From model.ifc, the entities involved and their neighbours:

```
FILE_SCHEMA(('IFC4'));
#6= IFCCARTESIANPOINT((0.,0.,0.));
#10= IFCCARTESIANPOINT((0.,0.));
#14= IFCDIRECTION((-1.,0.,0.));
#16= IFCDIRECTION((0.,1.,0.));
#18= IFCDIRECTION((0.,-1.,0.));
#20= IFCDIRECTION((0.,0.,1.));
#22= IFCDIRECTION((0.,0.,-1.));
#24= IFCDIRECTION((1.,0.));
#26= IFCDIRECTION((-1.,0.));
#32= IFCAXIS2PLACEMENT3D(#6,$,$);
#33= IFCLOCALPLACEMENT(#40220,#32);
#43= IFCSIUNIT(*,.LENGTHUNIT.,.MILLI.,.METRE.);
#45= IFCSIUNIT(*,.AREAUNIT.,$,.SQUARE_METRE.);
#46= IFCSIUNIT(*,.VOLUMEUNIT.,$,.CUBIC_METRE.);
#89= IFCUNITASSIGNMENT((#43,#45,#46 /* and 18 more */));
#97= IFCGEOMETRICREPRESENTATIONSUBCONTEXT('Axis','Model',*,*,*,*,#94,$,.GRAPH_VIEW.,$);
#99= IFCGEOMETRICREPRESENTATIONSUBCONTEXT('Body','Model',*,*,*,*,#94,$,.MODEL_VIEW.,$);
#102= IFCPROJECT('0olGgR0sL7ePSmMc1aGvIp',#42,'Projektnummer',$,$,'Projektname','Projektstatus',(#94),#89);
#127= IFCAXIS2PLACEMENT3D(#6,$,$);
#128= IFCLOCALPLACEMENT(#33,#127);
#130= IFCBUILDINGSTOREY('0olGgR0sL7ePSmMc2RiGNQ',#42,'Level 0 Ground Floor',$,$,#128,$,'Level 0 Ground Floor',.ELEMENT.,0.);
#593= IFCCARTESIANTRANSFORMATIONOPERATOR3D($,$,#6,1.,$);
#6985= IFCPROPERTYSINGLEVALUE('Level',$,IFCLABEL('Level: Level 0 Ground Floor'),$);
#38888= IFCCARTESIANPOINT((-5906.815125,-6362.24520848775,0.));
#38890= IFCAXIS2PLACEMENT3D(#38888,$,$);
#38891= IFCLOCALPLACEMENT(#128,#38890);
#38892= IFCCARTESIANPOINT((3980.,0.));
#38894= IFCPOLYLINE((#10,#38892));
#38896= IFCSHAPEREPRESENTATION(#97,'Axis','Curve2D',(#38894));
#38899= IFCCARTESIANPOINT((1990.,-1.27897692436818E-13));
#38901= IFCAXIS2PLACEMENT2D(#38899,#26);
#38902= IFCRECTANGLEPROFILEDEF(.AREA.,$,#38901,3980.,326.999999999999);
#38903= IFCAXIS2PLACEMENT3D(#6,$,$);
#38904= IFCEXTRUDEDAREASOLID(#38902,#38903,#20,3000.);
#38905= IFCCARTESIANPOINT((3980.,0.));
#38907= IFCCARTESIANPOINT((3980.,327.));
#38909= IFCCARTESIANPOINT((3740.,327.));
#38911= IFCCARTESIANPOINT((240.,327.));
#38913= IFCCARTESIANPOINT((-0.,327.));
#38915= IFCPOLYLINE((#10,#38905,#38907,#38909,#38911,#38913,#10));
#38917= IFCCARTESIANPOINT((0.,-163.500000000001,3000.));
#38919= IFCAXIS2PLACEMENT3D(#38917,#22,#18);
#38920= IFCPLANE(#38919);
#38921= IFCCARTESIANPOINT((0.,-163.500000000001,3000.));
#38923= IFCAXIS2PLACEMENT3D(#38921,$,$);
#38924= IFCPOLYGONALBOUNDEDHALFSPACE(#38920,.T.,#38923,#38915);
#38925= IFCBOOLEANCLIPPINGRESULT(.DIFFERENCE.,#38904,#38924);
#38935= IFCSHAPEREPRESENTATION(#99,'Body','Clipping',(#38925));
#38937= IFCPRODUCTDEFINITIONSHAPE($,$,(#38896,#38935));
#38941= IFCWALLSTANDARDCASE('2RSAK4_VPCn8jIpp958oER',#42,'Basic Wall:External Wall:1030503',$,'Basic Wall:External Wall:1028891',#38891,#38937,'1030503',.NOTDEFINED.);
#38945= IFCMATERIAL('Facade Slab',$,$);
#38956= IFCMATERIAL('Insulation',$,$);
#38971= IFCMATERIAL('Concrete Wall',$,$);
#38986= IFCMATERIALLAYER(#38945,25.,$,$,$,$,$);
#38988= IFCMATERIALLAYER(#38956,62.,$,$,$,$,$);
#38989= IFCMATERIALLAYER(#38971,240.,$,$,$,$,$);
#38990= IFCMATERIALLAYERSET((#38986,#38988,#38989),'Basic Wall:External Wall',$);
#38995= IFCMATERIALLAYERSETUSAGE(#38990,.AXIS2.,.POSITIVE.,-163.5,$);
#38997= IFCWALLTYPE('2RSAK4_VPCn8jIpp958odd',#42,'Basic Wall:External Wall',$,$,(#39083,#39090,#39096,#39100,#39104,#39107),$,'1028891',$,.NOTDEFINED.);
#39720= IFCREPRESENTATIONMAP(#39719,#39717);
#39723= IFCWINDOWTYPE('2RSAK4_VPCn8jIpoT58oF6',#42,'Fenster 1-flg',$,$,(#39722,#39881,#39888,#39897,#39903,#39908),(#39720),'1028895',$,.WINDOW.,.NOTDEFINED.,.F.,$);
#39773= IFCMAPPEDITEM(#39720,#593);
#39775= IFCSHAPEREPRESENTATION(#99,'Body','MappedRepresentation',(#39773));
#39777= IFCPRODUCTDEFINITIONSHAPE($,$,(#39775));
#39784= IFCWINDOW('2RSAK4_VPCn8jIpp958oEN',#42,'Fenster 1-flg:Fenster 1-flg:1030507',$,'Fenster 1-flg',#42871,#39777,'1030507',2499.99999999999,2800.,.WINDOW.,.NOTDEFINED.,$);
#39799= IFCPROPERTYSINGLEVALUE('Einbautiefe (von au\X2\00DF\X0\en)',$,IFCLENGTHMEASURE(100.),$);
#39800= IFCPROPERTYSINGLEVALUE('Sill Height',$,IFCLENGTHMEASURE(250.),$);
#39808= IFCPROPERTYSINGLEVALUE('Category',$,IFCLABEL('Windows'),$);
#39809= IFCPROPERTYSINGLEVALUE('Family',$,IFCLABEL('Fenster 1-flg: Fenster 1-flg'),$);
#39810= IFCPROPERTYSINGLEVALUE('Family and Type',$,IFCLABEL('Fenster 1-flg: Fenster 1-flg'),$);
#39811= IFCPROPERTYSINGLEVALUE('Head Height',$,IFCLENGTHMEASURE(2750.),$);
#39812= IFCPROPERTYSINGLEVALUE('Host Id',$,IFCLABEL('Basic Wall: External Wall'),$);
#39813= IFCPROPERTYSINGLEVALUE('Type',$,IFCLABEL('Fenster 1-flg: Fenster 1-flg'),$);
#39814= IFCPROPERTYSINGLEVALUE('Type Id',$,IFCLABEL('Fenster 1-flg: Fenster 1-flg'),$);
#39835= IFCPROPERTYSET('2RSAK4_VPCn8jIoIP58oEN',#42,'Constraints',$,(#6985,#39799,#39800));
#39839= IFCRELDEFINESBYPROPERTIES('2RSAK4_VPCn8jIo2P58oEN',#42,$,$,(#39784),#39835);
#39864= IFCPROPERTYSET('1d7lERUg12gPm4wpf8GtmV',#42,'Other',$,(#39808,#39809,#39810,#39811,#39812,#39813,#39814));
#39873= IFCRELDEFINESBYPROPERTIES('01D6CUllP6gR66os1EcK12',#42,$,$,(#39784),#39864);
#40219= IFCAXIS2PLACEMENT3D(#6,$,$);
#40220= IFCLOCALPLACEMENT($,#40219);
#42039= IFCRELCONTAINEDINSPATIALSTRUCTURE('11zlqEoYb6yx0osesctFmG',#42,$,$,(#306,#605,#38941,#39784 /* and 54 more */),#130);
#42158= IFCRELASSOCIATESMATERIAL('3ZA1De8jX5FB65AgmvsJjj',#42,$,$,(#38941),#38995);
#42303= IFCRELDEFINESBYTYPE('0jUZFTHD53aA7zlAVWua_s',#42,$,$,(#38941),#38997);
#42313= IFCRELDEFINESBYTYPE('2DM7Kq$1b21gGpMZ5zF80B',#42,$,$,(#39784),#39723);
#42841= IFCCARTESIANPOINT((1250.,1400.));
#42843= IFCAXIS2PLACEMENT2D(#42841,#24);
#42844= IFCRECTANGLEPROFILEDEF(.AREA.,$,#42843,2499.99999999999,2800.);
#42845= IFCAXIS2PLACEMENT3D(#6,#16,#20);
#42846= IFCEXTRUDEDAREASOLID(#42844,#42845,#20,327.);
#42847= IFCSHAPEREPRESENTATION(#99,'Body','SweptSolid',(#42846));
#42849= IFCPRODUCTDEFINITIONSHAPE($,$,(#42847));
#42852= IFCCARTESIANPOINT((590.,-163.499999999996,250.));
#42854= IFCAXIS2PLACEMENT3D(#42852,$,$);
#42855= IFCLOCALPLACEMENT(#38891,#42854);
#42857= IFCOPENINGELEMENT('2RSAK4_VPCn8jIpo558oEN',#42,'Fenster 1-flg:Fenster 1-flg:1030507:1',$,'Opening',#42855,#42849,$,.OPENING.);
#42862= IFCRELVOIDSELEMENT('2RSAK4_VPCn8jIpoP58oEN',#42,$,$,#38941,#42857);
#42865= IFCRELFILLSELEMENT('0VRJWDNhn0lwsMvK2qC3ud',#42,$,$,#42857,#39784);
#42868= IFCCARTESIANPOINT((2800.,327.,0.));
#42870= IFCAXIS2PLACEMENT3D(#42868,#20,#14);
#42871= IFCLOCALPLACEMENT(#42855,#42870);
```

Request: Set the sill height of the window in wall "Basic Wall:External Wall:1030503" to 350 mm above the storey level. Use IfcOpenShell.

```python
import numpy as np
import ifcopenshell
import ifcopenshell.api.geometry
import ifcopenshell.api.pset
import ifcopenshell.geom
import ifcopenshell.util.element
import ifcopenshell.util.placement
import ifcopenshell.util.shape
import ifcopenshell.util.unit

model = ifcopenshell.open("model.ifc")
unit_scale = ifcopenshell.util.unit.calculate_unit_scale(model)

window = model.by_guid("2RSAK4_VPCn8jIpp958oEN")
opening = window.FillsVoids[0].RelatingOpeningElement
storey = ifcopenshell.util.element.get_container(window, ifc_class="IfcBuildingStorey")
level = ifcopenshell.util.placement.get_local_placement(storey.ObjectPlacement)[2, 3]

# The opening's origin need not be at the sill, so measure its lowest point.
shape = ifcopenshell.geom.create_shape(ifcopenshell.geom.settings(), opening)
bottom = ifcopenshell.util.shape.get_shape_bottom_elevation(shape, shape.geometry) / unit_scale
dz = level + 0.35 / unit_scale - bottom

shift = np.array([0.0, 0.0, dz])
# The window is placed relative to its opening, so it follows when the opening moves.
matrix = ifcopenshell.util.placement.get_local_placement(opening.ObjectPlacement)
matrix[:3, 3] += shift
ifcopenshell.api.geometry.edit_object_placement(
    model, product=opening, matrix=matrix, is_si=False, should_transform_children=True
)

# Keep the stored heights in step.
pset = model.by_id(ifcopenshell.util.element.get_pset(window, "Constraints", should_inherit=False)["id"])
ifcopenshell.api.pset.edit_pset(model, pset=pset, properties={
    "Sill Height": model.create_entity("IfcLengthMeasure", ifcopenshell.util.element.get_pset(window, "Constraints", "Sill Height") + dz),
})
pset = model.by_id(ifcopenshell.util.element.get_pset(window, "Other", should_inherit=False)["id"])
ifcopenshell.api.pset.edit_pset(model, pset=pset, properties={
    "Head Height": model.create_entity("IfcLengthMeasure", ifcopenshell.util.element.get_pset(window, "Other", "Head Height") + dz),
})

print(f"moved by {dz * unit_scale:+.3f} m")

model.write("model_updated.ifc")
```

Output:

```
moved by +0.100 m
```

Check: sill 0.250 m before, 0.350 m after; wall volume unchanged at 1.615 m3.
